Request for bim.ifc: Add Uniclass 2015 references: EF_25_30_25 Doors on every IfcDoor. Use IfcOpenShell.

First a look at what the model holds.

```python
import ifcopenshell

model = ifcopenshell.open("bim.ifc")
print(model.schema)
print("classifications:", [c.Name for c in model.by_type("IfcClassification")])
for ifc_class in ("IfcDoor", "IfcRoof", "IfcStair", "IfcWall", "IfcWindow"):
    print(ifc_class, len(model.by_type(ifc_class)))
```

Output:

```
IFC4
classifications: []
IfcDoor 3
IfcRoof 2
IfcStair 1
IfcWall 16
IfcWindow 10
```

```python
import ifcopenshell
import ifcopenshell.api.classification

model = ifcopenshell.open("bim.ifc")

system = ifcopenshell.api.classification.add_classification(model, classification="Uniclass 2015")

codes = {
    "IfcDoor": ("EF_25_30_25", "Doors"),
}
for ifc_class, (code, name) in codes.items():
    products = model.by_type(ifc_class)
    ifcopenshell.api.classification.add_reference(
        model, products=products, classification=system, identification=code, name=name
    )
    print(code, len(products))

model.write("bim_v2.ifc")
```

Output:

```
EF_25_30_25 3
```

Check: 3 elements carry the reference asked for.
